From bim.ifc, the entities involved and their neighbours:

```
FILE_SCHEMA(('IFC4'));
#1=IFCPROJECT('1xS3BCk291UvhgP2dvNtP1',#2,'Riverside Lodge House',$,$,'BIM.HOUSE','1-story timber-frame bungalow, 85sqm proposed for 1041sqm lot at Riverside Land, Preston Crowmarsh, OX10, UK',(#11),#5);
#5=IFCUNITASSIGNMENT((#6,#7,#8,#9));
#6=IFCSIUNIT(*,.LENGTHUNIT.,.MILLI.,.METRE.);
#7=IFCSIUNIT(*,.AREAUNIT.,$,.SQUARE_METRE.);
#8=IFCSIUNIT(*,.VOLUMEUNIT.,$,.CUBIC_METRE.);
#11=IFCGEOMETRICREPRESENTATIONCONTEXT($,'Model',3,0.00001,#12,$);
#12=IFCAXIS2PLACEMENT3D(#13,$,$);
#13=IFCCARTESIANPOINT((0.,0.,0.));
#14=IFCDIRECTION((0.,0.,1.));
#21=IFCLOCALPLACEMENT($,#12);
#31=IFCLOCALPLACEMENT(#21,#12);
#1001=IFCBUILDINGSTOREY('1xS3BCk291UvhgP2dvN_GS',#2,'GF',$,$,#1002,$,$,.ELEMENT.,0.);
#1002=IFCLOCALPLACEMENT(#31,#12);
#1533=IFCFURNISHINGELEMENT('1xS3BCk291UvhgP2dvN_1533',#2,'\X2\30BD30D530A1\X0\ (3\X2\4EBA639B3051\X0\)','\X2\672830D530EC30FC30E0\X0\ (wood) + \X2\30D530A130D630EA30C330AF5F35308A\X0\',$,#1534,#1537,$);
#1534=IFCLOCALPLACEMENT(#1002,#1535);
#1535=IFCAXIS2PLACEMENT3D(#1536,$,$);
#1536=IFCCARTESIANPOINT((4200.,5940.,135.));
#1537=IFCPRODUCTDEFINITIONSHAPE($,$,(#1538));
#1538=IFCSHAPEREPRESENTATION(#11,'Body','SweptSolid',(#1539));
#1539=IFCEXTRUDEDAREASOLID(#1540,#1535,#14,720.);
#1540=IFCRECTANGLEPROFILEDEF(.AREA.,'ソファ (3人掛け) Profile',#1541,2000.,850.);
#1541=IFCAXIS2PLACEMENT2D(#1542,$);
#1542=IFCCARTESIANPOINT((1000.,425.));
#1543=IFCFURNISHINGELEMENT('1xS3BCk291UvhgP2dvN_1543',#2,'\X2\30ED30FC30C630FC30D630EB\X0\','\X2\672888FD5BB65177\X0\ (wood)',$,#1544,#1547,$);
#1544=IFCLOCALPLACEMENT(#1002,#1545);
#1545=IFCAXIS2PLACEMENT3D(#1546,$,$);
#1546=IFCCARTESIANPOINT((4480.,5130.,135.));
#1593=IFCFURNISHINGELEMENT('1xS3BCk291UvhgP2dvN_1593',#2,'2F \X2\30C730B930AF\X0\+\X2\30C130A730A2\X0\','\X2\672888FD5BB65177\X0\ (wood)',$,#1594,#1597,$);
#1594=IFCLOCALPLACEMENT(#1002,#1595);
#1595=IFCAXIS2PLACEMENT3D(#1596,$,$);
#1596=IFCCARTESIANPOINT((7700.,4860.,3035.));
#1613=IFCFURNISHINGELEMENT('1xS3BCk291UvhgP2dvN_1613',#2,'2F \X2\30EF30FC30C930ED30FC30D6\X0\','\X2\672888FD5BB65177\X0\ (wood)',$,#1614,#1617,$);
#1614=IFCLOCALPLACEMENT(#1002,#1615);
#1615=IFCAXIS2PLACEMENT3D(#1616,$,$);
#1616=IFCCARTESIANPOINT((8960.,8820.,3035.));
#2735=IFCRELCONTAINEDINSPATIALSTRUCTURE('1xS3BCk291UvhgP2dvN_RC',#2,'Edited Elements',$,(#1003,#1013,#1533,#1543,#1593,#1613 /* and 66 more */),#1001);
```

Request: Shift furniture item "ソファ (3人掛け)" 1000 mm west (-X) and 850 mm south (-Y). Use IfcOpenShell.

```python
import ifcopenshell
import ifcopenshell.api.geometry
import ifcopenshell.util.placement

model = ifcopenshell.open("bim.ifc")

item = model.by_id(1533)
matrix = ifcopenshell.util.placement.get_local_placement(item.ObjectPlacement)
matrix[0, 3] -= 1000.0
matrix[1, 3] -= 850.0
ifcopenshell.api.geometry.edit_object_placement(model, product=item, matrix=matrix, is_si=False)

print(ifcopenshell.util.placement.get_local_placement(item.ObjectPlacement).round(3) + 0.0)

model.write("bim-out.ifc")
```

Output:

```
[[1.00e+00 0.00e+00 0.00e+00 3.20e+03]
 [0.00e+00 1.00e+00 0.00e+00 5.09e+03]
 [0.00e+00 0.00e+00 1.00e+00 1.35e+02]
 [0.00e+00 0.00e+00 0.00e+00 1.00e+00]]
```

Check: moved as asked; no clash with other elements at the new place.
